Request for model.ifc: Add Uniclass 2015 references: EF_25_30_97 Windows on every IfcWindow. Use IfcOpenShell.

First a look at what the model holds.

```python
import ifcopenshell

model = ifcopenshell.open("model.ifc")
print(model.schema)
print("classifications:", [c.Name for c in model.by_type("IfcClassification")])
for ifc_class in ("IfcDoor", "IfcRoof", "IfcStair", "IfcWall", "IfcWindow"):
    print(ifc_class, len(model.by_type(ifc_class)))
```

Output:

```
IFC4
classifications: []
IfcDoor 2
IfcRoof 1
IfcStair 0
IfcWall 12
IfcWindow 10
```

```python
import ifcopenshell
import ifcopenshell.api.classification

model = ifcopenshell.open("model.ifc")

system = ifcopenshell.api.classification.add_classification(model, classification="Uniclass 2015")

codes = {
    "IfcWindow": ("EF_25_30_97", "Windows"),
}
for ifc_class, (code, name) in codes.items():
    products = model.by_type(ifc_class)
    ifcopenshell.api.classification.add_reference(
        model, products=products, classification=system, identification=code, name=name
    )
    print(code, len(products))

model.write("model_rev.ifc")
```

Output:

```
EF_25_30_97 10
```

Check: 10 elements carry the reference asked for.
